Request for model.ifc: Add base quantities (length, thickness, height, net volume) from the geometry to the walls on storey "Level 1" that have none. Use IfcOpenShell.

First a look at what the model holds.

```python
import ifcopenshell
import ifcopenshell.util.element
import ifcopenshell.util.unit

model = ifcopenshell.open("model.ifc")
print(model.schema)
for unit_type in ("LENGTHUNIT", "AREAUNIT", "VOLUMEUNIT"):
    print(unit_type, ifcopenshell.util.unit.calculate_unit_scale(model, unit_type))
storey = next(s for s in model.by_type("IfcBuildingStorey") if s.Name == "Level 1")
walls = [e for e in ifcopenshell.util.element.get_decomposition(storey) if e.is_a("IfcWall")]
for e in sorted(walls, key=lambda e: e.id()):
    print(e.id(), e.is_a(), e.Name, list(ifcopenshell.util.element.get_psets(e, qtos_only=True)), sep=" | ")
```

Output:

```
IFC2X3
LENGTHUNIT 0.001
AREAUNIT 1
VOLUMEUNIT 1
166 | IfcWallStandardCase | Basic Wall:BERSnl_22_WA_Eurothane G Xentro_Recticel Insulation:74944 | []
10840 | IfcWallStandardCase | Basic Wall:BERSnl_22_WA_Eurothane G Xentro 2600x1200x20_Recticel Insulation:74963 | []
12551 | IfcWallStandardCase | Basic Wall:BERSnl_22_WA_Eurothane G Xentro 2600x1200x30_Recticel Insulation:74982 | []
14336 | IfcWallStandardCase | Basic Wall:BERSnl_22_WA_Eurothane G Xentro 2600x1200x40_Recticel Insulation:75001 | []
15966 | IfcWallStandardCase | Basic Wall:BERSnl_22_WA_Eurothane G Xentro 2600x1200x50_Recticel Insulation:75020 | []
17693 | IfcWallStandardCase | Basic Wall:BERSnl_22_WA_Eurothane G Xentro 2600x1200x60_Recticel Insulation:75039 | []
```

```python
import ifcopenshell
import ifcopenshell.api.pset
import ifcopenshell.geom
import ifcopenshell.util.element
import ifcopenshell.util.shape
import ifcopenshell.util.unit

model = ifcopenshell.open("model.ifc")
unit_scale = ifcopenshell.util.unit.calculate_unit_scale(model)
volume_scale = ifcopenshell.util.unit.calculate_unit_scale(model, "VOLUMEUNIT")
settings = ifcopenshell.geom.settings()

storey = next(s for s in model.by_type("IfcBuildingStorey") if s.Name == "Level 1")
walls = [e for e in ifcopenshell.util.element.get_decomposition(storey) if e.is_a("IfcWall")]

for e in sorted(walls, key=lambda e: e.id()):
    if ifcopenshell.util.element.get_psets(e, qtos_only=True, should_inherit=False):
        continue
    # Geometry comes back in metres, in the element's own axes.
    shape = ifcopenshell.geom.create_shape(settings, e)
    values = {
        "Length": ifcopenshell.util.shape.get_x(shape.geometry) / unit_scale,
        "Width": ifcopenshell.util.shape.get_y(shape.geometry) / unit_scale,
        "Height": ifcopenshell.util.shape.get_z(shape.geometry) / unit_scale,
        "NetVolume": ifcopenshell.util.shape.get_volume(shape.geometry) / volume_scale,
    }
    qto = ifcopenshell.api.pset.add_qto(model, product=e, name="BaseQuantities")
    ifcopenshell.api.pset.edit_qto(model, qto=qto, properties=values)
    print(e.id(), {k: round(v, 3) for k, v in values.items()})

model.write("model_edited.ifc")
```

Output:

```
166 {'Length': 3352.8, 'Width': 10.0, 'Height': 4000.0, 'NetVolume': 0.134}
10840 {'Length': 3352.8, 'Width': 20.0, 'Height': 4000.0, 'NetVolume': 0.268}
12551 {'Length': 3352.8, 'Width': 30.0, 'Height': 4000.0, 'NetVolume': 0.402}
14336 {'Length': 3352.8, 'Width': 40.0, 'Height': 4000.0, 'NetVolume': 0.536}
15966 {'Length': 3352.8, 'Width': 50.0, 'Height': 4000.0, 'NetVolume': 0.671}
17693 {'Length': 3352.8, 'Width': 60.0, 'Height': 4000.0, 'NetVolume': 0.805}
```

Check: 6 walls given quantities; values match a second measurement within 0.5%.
